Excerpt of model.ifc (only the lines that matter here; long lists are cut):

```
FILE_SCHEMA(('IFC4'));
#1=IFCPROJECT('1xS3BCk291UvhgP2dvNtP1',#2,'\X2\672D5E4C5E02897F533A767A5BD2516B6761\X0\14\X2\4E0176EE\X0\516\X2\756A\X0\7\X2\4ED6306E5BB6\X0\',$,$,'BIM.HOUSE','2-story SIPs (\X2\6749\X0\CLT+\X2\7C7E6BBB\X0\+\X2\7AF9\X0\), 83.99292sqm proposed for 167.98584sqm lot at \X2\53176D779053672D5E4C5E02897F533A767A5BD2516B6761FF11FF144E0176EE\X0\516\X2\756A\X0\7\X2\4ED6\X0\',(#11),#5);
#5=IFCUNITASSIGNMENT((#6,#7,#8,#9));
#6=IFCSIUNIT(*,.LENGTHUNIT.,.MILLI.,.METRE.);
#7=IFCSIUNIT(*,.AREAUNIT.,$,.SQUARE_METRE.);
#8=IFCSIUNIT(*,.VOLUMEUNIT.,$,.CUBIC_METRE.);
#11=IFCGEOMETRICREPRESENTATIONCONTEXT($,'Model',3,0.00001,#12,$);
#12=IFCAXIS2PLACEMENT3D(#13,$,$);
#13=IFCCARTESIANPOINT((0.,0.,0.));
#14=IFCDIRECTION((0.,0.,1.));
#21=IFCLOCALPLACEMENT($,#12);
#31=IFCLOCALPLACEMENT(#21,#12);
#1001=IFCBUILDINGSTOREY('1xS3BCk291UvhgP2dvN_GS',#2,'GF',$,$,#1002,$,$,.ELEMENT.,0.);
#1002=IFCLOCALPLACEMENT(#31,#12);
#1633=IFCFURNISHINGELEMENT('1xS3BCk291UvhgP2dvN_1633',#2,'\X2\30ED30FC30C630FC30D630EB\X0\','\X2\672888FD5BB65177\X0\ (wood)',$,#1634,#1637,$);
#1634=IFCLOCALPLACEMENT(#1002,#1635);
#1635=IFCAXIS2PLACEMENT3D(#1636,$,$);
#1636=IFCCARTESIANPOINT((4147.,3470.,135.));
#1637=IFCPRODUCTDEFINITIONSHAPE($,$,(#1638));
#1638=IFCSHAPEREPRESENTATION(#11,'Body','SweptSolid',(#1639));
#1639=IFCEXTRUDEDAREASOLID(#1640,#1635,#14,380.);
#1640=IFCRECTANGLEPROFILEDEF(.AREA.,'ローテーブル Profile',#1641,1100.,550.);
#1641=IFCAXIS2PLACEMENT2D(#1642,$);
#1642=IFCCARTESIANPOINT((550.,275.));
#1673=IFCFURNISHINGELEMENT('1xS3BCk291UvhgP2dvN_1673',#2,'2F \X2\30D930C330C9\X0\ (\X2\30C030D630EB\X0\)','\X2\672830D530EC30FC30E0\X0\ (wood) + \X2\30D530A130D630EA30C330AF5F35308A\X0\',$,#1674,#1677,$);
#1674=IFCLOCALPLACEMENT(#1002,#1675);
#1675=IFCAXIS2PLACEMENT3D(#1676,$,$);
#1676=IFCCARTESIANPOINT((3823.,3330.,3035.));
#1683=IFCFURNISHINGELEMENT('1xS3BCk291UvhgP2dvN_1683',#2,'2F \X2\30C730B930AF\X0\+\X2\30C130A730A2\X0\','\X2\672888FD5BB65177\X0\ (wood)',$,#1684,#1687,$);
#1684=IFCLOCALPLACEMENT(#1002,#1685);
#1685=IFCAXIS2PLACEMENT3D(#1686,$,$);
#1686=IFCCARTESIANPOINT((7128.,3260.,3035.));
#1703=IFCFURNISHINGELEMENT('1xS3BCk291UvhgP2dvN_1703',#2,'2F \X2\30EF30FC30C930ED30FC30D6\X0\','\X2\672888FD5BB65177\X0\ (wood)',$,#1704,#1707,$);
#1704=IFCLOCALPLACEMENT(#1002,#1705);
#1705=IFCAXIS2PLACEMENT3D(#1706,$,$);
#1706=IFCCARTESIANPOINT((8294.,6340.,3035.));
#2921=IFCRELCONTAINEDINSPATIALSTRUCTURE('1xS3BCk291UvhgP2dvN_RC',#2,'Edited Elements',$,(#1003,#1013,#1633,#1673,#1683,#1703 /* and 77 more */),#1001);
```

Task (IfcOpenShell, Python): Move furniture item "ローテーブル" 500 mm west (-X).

```python
import ifcopenshell
import ifcopenshell.api.geometry
import ifcopenshell.util.placement
import ifcopenshell.util.unit

model = ifcopenshell.open("model.ifc")
unit_scale = ifcopenshell.util.unit.calculate_unit_scale(model)

item = model.by_guid("1xS3BCk291UvhgP2dvN_1633")
matrix = ifcopenshell.util.placement.get_local_placement(item.ObjectPlacement)
matrix[0, 3] -= 0.5 / unit_scale
ifcopenshell.api.geometry.edit_object_placement(model, product=item, matrix=matrix, is_si=False)

print(ifcopenshell.util.placement.get_local_placement(item.ObjectPlacement).round(3) + 0.0)

model.write("model-out.ifc")
```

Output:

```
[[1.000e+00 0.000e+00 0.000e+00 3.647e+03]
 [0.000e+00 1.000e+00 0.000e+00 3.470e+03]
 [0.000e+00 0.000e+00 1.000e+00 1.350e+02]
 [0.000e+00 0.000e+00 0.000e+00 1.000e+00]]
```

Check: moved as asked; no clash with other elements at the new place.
